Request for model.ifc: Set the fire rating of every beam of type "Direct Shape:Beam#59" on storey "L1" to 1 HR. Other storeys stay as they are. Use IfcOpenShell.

First a look at what the model holds.

```python
import ifcopenshell
import ifcopenshell.util.element

model = ifcopenshell.open("model.ifc")
print(model.schema)
storey = next(s for s in model.by_type("IfcBuildingStorey") if s.Name == "L1")
beams = [e for e in ifcopenshell.util.element.get_decomposition(storey) if e.is_a("IfcBeam")]
seen = {}
for e in beams:
    element_type = ifcopenshell.util.element.get_type(e)
    key = (element_type.Name if element_type != e and element_type else None, ifcopenshell.util.element.get_pset(e, "Pset_BeamCommon", "FireRating"))
    seen[key] = seen.get(key, 0) + 1
for (name, value), count in sorted(seen.items(), key=str):
    print(count, "x", name, "|", value)
```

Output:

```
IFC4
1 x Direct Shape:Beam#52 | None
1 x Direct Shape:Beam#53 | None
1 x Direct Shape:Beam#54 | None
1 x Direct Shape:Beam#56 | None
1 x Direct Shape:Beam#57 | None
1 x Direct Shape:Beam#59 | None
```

```python
import ifcopenshell
import ifcopenshell.api.pset
import ifcopenshell.util.element

model = ifcopenshell.open("model.ifc")

storey = next(s for s in model.by_type("IfcBuildingStorey") if s.Name == "L1")
beams = [e for e in ifcopenshell.util.element.get_decomposition(storey) if e.is_a("IfcBeam")]

count = 0
for e in beams:
    element_type = ifcopenshell.util.element.get_type(e)
    if element_type in (None, e) or element_type.Name != "Direct Shape:Beam#59":
        continue
    # add_pset returns the element's existing set when there is one.
    pset = ifcopenshell.api.pset.add_pset(model, product=e, name="Pset_BeamCommon")
    ifcopenshell.api.pset.edit_pset(model, pset=pset, properties={"FireRating": "1 HR"})
    count += 1

print(count, "beams updated")

model.write("model_edited.ifc")
```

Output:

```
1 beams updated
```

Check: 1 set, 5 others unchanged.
